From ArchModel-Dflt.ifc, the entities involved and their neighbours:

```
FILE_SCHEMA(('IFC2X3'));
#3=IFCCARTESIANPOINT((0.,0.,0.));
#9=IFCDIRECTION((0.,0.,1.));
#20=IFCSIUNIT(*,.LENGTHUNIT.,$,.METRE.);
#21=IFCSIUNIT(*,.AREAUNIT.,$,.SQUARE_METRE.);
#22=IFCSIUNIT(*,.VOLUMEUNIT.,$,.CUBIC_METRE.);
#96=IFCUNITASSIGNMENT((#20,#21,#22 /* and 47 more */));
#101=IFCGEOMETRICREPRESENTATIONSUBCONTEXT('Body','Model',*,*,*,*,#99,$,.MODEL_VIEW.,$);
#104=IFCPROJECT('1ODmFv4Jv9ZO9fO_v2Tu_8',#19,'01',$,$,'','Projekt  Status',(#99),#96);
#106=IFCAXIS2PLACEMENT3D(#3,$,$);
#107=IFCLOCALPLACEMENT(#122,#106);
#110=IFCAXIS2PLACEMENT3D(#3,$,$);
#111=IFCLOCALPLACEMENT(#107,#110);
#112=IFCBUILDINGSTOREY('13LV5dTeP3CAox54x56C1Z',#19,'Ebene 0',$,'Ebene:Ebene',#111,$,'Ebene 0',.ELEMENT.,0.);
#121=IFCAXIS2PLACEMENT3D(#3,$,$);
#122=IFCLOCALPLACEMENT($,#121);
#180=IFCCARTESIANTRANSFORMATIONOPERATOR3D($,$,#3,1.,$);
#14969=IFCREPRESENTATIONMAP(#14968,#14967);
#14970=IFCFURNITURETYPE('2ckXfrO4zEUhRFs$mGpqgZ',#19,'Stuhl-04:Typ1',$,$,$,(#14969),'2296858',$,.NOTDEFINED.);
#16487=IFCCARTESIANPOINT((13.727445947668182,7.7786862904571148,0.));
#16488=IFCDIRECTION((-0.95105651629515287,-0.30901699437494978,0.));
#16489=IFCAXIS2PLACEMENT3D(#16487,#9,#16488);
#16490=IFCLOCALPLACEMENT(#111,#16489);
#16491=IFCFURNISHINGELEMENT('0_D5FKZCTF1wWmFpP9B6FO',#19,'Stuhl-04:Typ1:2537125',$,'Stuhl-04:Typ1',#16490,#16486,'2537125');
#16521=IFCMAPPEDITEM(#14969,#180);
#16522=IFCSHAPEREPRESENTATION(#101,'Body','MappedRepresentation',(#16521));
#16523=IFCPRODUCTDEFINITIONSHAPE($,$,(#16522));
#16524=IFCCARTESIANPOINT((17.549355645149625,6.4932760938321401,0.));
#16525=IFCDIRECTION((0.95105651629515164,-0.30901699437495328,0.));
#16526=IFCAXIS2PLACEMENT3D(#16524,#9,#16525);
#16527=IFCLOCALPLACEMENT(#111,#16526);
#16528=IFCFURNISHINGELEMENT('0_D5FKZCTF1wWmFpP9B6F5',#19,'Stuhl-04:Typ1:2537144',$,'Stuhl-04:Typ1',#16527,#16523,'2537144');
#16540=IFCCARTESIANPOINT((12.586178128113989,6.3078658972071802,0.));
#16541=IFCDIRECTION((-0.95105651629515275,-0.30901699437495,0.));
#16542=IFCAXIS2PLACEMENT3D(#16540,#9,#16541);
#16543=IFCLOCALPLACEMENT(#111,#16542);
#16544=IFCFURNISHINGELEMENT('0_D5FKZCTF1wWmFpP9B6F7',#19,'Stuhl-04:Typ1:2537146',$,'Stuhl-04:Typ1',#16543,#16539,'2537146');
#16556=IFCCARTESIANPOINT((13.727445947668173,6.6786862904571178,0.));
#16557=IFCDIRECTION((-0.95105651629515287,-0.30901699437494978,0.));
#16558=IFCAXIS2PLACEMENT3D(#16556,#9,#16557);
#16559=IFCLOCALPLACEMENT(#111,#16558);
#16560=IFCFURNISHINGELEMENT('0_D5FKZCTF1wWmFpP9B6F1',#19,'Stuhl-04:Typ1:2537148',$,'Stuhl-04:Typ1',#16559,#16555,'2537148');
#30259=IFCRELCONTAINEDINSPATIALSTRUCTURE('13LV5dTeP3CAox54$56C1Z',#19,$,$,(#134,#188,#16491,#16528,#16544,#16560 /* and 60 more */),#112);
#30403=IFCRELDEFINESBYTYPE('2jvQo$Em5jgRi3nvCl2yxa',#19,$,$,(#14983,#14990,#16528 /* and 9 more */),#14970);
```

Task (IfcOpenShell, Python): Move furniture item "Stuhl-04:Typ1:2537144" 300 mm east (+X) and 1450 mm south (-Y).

```python
import ifcopenshell
import ifcopenshell.api.geometry
import ifcopenshell.util.placement

model = ifcopenshell.open("ArchModel-Dflt.ifc")

item = model.by_id(16528)
matrix = ifcopenshell.util.placement.get_local_placement(item.ObjectPlacement)
matrix[0, 3] += 0.3
matrix[1, 3] -= 1.45
ifcopenshell.api.geometry.edit_object_placement(model, product=item, matrix=matrix, is_si=False)

print(ifcopenshell.util.placement.get_local_placement(item.ObjectPlacement).round(3) + 0.0)

model.write("ArchModel-Dflt_updated.ifc")
```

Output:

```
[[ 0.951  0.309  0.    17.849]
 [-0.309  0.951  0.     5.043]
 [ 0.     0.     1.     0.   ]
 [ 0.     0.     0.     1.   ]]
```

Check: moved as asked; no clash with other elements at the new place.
